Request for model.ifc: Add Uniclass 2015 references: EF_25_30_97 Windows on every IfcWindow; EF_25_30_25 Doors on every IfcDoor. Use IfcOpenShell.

First a look at what the model holds.

```python
import ifcopenshell

model = ifcopenshell.open("model.ifc")
print(model.schema)
print("classifications:", [c.Name for c in model.by_type("IfcClassification")])
for ifc_class in ("IfcDoor", "IfcRoof", "IfcStair", "IfcWall", "IfcWindow"):
    print(ifc_class, len(model.by_type(ifc_class)))
```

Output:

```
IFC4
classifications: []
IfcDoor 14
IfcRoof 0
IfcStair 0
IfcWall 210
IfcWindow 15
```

```python
import ifcopenshell
import ifcopenshell.api.classification

model = ifcopenshell.open("model.ifc")

system = ifcopenshell.api.classification.add_classification(model, classification="Uniclass 2015")

codes = {
    "IfcWindow": ("EF_25_30_97", "Windows"),
    "IfcDoor": ("EF_25_30_25", "Doors"),
}
for ifc_class, (code, name) in codes.items():
    products = model.by_type(ifc_class)
    ifcopenshell.api.classification.add_reference(
        model, products=products, classification=system, identification=code, name=name
    )
    print(code, len(products))

model.write("model_v2.ifc")
```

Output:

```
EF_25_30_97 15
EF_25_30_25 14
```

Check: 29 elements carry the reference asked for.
